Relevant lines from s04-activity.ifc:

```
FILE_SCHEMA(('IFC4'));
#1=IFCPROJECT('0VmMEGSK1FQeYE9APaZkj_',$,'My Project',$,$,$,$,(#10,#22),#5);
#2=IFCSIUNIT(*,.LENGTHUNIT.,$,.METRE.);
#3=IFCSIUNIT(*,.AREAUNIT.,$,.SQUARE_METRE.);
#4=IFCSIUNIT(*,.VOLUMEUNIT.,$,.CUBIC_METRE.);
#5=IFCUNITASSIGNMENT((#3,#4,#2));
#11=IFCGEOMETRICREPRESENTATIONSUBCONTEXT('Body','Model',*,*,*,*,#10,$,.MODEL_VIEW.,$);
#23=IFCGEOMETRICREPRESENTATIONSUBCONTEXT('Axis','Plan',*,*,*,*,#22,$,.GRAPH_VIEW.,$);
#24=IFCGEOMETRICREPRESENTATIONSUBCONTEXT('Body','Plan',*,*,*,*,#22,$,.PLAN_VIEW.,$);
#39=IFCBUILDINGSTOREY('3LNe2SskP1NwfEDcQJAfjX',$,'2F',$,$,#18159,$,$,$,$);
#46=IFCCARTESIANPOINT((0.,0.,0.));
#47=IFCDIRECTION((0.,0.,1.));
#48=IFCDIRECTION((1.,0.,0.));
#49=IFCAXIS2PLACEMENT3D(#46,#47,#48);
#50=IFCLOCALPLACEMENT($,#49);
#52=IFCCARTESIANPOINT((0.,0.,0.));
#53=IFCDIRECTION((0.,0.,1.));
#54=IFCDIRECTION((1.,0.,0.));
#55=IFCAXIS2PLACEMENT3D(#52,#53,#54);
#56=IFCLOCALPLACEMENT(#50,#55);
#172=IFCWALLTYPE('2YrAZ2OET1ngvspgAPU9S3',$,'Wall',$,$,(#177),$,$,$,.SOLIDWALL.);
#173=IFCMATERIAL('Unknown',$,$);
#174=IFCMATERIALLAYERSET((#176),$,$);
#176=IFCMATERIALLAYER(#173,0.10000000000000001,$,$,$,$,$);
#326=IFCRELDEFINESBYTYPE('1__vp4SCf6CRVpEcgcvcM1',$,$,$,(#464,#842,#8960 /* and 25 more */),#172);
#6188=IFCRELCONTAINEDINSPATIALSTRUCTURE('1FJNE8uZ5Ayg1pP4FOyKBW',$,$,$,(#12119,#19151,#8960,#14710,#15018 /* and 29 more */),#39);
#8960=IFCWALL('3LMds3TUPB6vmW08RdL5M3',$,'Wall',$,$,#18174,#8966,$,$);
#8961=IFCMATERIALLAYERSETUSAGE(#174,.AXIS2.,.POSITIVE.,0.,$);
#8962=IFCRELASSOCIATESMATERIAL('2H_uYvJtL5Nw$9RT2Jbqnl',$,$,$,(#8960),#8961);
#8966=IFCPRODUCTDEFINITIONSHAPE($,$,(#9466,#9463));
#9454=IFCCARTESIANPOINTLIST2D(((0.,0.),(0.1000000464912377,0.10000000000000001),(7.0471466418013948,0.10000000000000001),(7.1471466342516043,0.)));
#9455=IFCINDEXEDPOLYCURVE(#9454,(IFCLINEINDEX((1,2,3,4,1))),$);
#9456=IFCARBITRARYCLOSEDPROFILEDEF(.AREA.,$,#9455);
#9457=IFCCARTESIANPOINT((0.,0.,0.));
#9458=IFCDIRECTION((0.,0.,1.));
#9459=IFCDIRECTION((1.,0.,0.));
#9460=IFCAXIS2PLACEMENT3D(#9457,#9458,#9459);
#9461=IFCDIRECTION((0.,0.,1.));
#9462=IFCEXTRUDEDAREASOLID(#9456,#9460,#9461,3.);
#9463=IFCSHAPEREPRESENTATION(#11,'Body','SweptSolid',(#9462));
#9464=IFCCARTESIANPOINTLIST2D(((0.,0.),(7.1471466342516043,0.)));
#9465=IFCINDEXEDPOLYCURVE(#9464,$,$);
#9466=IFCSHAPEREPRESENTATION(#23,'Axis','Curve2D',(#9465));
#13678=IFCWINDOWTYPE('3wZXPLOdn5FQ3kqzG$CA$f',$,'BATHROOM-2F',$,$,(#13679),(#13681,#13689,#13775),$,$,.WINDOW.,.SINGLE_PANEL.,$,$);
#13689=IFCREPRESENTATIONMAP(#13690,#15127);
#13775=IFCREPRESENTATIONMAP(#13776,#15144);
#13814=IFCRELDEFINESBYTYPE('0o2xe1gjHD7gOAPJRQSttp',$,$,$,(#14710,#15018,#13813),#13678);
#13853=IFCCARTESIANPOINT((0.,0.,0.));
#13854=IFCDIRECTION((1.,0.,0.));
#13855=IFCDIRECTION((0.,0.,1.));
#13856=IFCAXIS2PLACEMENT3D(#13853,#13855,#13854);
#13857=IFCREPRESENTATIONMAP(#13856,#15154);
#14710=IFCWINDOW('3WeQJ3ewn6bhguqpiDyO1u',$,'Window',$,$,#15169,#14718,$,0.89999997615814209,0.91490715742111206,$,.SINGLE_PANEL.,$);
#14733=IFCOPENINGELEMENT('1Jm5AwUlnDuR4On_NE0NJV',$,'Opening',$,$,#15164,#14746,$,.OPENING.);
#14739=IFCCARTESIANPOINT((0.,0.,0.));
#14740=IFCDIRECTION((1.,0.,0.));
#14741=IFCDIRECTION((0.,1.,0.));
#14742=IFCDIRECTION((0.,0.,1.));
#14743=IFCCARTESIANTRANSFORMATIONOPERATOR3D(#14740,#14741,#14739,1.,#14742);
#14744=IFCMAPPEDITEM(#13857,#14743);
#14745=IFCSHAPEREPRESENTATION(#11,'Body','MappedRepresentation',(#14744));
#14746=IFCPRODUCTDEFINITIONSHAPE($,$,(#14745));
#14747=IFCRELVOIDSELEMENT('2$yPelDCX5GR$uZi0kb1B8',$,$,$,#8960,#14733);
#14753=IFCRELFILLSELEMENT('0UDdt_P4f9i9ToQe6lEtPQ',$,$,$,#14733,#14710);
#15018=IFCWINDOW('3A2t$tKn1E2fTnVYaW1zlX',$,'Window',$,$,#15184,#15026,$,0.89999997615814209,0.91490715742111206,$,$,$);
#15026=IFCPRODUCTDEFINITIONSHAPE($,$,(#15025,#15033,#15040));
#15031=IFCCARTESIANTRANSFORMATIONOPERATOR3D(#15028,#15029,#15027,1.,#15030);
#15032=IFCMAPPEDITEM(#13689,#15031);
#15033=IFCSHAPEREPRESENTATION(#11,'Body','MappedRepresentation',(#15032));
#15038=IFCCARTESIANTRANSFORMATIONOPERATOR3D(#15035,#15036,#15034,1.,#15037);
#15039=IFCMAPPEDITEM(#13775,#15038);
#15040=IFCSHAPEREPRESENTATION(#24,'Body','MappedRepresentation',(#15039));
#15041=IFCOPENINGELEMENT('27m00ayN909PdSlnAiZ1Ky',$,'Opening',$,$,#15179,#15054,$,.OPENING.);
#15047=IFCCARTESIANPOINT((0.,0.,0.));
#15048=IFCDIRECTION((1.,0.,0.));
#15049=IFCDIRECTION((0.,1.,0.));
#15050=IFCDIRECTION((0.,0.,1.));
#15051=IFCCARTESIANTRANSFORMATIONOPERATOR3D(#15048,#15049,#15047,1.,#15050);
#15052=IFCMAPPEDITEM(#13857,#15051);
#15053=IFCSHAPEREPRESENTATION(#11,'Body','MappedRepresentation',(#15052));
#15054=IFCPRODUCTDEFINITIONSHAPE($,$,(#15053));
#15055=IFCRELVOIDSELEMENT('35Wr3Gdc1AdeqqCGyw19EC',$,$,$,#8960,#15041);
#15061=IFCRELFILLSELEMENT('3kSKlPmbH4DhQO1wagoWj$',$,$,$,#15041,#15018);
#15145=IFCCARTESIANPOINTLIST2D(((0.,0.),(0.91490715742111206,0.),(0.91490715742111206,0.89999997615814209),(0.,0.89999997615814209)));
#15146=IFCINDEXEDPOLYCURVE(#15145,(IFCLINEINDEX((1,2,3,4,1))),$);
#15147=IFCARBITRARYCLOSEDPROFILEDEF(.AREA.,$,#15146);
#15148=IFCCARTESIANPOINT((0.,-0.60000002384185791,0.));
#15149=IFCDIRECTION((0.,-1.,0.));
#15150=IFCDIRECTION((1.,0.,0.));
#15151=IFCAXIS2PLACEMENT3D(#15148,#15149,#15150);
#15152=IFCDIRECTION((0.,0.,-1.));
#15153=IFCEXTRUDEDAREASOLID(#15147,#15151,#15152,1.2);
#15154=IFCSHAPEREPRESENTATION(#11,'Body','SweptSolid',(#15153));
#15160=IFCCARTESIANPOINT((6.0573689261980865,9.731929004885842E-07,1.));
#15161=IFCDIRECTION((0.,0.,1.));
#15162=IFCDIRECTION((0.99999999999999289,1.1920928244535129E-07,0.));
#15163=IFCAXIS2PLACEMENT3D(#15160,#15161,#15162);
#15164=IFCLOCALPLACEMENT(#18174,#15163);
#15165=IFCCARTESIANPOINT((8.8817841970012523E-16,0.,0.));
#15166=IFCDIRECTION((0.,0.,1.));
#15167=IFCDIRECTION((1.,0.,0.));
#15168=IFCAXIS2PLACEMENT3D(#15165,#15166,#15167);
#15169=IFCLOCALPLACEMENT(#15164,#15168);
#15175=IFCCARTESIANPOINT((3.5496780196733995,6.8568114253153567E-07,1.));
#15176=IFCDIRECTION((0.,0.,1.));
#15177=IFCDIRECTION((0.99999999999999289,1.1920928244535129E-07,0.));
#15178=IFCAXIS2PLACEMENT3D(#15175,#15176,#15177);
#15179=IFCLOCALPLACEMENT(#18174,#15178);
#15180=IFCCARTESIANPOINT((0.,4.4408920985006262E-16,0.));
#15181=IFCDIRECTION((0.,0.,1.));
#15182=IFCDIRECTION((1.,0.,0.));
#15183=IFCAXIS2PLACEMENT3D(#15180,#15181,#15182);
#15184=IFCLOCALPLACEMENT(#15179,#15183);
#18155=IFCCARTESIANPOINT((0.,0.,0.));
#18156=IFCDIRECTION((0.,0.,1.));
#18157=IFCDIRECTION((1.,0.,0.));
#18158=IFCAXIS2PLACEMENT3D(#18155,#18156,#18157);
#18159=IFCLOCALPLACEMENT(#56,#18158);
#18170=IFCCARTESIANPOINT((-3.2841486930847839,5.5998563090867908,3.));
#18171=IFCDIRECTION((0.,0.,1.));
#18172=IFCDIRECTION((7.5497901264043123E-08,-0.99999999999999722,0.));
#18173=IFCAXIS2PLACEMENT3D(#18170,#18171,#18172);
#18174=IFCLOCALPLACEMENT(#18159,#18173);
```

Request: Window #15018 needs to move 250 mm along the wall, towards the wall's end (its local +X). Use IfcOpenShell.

```python
import ifcopenshell
import ifcopenshell.api.geometry
import ifcopenshell.util.placement
import ifcopenshell.util.unit

model = ifcopenshell.open("s04-activity.ifc")
unit_scale = ifcopenshell.util.unit.calculate_unit_scale(model)

window = model.by_id(15018)
opening = window.FillsVoids[0].RelatingOpeningElement
wall = opening.VoidsElements[0].RelatingBuildingElement

wall_matrix = ifcopenshell.util.placement.get_local_placement(wall.ObjectPlacement)
shift = wall_matrix[:3, 0] * 0.25 / unit_scale
before = ifcopenshell.util.placement.get_local_placement(window.ObjectPlacement)[:3, 3].copy()

# The window is placed relative to its opening, so it follows when the opening moves.
matrix = ifcopenshell.util.placement.get_local_placement(opening.ObjectPlacement)
matrix[:3, 3] += shift
ifcopenshell.api.geometry.edit_object_placement(
    model, product=opening, matrix=matrix, is_si=False, should_transform_children=True
)

after = ifcopenshell.util.placement.get_local_placement(window.ObjectPlacement)[:3, 3]
print("window moved by", (after - before).round(3) + 0.0)

model.write("s04-activity-out.ifc")
```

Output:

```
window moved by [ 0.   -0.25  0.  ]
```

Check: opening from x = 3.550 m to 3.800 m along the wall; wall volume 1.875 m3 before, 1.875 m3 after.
